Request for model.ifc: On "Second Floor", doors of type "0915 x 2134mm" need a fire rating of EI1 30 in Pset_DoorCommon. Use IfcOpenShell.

First a look at what the model holds.

```python
import ifcopenshell
import ifcopenshell.util.element

model = ifcopenshell.open("model.ifc")
print(model.schema)
storey = next(s for s in model.by_type("IfcBuildingStorey") if s.Name == "Second Floor")
doors = [e for e in ifcopenshell.util.element.get_decomposition(storey) if e.is_a("IfcDoor")]
seen = {}
for e in doors:
    element_type = ifcopenshell.util.element.get_type(e)
    key = (element_type.Name if element_type != e and element_type else None, ifcopenshell.util.element.get_pset(e, "Pset_DoorCommon", "FireRating"))
    seen[key] = seen.get(key, 0) + 1
for (name, value), count in sorted(seen.items(), key=str):
    print(count, "x", name, "|", value)
```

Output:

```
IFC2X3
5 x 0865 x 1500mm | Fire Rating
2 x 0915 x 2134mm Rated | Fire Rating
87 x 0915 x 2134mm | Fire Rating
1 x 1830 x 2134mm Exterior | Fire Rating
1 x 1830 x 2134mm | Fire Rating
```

```python
import ifcopenshell
import ifcopenshell.api.pset
import ifcopenshell.util.element

model = ifcopenshell.open("model.ifc")

storey = next(s for s in model.by_type("IfcBuildingStorey") if s.Name == "Second Floor")
doors = [e for e in ifcopenshell.util.element.get_decomposition(storey) if e.is_a("IfcDoor")]

count = 0
for e in doors:
    element_type = ifcopenshell.util.element.get_type(e)
    if element_type in (None, e) or element_type.Name != "0915 x 2134mm":
        continue
    # add_pset returns the element's existing set when there is one.
    pset = ifcopenshell.api.pset.add_pset(model, product=e, name="Pset_DoorCommon")
    ifcopenshell.api.pset.edit_pset(model, pset=pset, properties={"FireRating": "EI1 30"})
    count += 1

print(count, "doors updated")

model.write("model-out.ifc")
```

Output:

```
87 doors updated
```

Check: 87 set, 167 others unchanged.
